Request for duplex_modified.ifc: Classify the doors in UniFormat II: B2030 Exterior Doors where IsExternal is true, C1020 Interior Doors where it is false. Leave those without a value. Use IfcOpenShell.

First a look at what the model holds.

```python
import ifcopenshell
import ifcopenshell.util.element

model = ifcopenshell.open("duplex_modified.ifc")
print(model.schema)
print("classifications:", [c.Name for c in model.by_type("IfcClassification")])
values = [ifcopenshell.util.element.get_pset(e, "Pset_DoorCommon", "IsExternal") for e in model.by_type("IfcDoor")]
for value in (True, False, None):
    print("IsExternal", value, values.count(value))
```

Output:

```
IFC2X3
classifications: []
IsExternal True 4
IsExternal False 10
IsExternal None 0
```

```python
import ifcopenshell
import ifcopenshell.api.classification
import ifcopenshell.util.element

model = ifcopenshell.open("duplex_modified.ifc")

# IFC2X3 requires Source and Edition and has no link from the project to the system.
system = model.create_entity("IfcClassification", Source="ASTM", Edition="E1557", Name="UniFormat II")

doors = model.by_type("IfcDoor")
external = {e: ifcopenshell.util.element.get_pset(e, "Pset_DoorCommon", "IsExternal") for e in doors}
for flag, code, name in ((True, "B2030", "Exterior Doors"), (False, "C1020", "Interior Doors")):
    products = [e for e in doors if external[e] is flag]
    ifcopenshell.api.classification.add_reference(
        model, products=products, classification=system, identification=code, name=name
    )
    print(code, len(products))

model.write("duplex_modified_v2.ifc")
```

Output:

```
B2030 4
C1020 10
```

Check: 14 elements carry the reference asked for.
